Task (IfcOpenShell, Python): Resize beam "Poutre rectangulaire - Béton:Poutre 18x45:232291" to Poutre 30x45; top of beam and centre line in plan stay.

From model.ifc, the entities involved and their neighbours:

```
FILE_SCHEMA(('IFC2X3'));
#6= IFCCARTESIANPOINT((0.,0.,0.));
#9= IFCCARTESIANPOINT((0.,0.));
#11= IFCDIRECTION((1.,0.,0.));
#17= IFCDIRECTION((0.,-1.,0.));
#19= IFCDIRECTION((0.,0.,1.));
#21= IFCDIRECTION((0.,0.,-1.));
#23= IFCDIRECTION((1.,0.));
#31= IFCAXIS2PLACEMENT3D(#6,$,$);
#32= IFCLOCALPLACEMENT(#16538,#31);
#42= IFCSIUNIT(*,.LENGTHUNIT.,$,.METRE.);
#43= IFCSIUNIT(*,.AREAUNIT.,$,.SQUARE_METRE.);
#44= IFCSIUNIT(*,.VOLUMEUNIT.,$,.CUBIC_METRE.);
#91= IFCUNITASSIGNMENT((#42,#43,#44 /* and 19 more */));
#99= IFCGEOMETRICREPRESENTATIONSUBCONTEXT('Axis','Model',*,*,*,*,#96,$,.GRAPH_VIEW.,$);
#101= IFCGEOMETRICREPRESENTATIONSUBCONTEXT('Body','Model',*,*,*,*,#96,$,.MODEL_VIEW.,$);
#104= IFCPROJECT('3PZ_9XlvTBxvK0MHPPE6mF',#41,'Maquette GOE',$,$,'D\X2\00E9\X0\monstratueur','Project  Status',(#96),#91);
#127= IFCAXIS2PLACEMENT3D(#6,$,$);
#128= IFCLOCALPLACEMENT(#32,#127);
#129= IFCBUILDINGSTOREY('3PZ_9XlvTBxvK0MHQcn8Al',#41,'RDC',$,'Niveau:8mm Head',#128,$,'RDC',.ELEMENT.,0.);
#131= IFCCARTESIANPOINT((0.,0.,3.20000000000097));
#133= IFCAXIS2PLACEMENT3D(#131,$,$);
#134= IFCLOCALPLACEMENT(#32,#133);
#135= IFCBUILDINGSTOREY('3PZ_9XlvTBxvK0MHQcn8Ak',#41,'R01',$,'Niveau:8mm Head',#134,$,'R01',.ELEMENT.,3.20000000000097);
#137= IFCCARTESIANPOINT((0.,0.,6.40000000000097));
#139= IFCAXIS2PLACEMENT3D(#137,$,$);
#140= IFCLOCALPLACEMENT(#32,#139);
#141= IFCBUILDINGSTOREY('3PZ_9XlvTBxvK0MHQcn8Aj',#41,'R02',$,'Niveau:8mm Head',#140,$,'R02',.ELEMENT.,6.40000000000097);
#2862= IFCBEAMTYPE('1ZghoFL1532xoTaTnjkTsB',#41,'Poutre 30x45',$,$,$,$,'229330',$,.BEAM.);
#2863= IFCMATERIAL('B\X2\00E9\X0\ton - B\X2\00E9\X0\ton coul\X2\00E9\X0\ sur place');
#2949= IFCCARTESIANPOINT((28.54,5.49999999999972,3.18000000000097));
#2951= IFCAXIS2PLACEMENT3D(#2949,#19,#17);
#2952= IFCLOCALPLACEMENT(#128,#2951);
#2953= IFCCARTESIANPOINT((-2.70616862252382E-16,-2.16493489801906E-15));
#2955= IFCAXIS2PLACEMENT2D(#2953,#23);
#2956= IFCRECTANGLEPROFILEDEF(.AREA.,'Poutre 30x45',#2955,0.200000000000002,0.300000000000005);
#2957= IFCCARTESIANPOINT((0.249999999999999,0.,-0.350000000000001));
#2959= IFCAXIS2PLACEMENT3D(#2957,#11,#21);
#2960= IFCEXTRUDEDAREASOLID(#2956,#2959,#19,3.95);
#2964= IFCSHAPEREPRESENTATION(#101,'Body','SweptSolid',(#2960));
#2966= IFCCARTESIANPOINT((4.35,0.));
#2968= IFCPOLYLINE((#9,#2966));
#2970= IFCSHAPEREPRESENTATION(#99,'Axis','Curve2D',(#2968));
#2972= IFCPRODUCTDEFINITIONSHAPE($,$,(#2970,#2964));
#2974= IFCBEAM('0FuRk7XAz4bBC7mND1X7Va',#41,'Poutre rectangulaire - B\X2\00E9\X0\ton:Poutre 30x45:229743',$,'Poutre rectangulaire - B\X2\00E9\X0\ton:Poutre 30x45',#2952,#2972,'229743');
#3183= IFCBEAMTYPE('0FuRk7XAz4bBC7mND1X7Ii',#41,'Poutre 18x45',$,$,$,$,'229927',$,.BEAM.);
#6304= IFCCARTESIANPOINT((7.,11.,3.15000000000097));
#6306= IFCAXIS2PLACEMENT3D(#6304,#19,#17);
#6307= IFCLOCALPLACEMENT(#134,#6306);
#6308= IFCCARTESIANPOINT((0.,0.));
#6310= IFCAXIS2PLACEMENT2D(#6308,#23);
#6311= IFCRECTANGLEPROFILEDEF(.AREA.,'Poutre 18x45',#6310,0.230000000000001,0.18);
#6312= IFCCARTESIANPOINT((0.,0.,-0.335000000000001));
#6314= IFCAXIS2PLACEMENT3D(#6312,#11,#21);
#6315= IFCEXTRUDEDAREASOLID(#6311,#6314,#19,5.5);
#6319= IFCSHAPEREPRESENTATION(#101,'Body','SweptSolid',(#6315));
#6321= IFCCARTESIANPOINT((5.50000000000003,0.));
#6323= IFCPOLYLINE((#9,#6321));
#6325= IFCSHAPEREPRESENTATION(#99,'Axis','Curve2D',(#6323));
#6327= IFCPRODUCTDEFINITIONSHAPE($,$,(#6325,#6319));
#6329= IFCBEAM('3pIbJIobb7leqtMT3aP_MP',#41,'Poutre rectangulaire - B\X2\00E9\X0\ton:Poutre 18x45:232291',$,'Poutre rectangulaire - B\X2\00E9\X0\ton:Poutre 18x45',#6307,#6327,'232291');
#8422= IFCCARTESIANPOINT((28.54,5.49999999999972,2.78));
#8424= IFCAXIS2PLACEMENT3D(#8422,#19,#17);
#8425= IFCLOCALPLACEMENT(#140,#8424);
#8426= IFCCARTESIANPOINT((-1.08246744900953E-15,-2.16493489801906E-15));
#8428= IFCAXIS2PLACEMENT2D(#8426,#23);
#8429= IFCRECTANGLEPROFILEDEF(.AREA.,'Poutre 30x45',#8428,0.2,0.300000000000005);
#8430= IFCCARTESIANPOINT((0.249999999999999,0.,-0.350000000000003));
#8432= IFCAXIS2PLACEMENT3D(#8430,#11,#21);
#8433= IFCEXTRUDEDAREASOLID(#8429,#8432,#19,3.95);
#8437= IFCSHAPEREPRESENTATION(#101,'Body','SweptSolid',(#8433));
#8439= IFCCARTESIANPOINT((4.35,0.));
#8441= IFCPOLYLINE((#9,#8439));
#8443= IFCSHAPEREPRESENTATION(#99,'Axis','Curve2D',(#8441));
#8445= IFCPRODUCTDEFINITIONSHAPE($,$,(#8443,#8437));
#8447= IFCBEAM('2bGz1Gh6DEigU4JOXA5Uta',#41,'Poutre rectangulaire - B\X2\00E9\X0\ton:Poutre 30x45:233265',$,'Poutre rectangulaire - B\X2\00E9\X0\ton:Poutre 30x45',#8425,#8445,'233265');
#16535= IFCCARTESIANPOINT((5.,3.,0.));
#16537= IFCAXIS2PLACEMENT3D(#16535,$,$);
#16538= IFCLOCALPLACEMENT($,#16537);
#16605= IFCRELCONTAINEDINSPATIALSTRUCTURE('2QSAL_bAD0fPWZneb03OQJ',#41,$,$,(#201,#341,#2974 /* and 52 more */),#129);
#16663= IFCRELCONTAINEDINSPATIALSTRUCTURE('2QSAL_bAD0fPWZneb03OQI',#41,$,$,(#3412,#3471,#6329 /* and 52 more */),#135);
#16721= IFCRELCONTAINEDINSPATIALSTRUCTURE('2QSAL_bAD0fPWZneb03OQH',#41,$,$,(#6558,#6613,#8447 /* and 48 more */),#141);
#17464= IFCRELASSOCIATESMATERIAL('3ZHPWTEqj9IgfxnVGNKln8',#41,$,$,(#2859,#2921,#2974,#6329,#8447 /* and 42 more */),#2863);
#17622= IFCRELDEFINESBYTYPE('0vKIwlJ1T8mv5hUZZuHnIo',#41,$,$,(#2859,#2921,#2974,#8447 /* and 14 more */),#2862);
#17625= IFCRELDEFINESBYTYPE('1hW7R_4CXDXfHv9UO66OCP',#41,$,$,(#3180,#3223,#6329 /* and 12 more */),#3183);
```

```python
import ifcopenshell
import ifcopenshell.api.type
import ifcopenshell.util.element
import ifcopenshell.util.representation

model = ifcopenshell.open("model.ifc")

member = model.by_guid("3pIbJIobb7leqtMT3aP_MP")
source = next(p for p in model.by_type("IfcRectangleProfileDef") if p.ProfileName == "Poutre 30x45")

body = ifcopenshell.util.representation.get_representation(member, "Model", "Body")
solid = body.Items[0]
old_profile = solid.SweptArea

# Copy the section's sizes but keep this member's own profile position.
profile = ifcopenshell.util.element.copy(model, source)
# Profiles are centred, so shift by half the change in depth to hold the top.
shift = (old_profile.XDim - profile.XDim) / 2
x, y = old_profile.Position.Location.Coordinates
up = (-1.0, 0.0)  # upwards, in the solid's own plane
location = model.createIfcCartesianPoint((x + up[0] * shift, y + up[1] * shift))
profile.Position = model.createIfcAxis2Placement2D(location, old_profile.Position.RefDirection)
solid.SweptArea = profile
if not model.get_total_inverses(old_profile):
    ifcopenshell.util.element.remove_deep2(model, old_profile)

new_type = model.by_guid("1ZghoFL1532xoTaTnjkTsB")
ifcopenshell.api.type.assign_type(
    model, related_objects=[member], relating_type=new_type, should_map_representations=False
)
member.Name = member.Name.replace("Poutre 18x45", "Poutre 30x45")
member.ObjectType = "Poutre rectangulaire - Béton:Poutre 30x45"

print(solid.SweptArea)

model.write("model_edited.ifc")
```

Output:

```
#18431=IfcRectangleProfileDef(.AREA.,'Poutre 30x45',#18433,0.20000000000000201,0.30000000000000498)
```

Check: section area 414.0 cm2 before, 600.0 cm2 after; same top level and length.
